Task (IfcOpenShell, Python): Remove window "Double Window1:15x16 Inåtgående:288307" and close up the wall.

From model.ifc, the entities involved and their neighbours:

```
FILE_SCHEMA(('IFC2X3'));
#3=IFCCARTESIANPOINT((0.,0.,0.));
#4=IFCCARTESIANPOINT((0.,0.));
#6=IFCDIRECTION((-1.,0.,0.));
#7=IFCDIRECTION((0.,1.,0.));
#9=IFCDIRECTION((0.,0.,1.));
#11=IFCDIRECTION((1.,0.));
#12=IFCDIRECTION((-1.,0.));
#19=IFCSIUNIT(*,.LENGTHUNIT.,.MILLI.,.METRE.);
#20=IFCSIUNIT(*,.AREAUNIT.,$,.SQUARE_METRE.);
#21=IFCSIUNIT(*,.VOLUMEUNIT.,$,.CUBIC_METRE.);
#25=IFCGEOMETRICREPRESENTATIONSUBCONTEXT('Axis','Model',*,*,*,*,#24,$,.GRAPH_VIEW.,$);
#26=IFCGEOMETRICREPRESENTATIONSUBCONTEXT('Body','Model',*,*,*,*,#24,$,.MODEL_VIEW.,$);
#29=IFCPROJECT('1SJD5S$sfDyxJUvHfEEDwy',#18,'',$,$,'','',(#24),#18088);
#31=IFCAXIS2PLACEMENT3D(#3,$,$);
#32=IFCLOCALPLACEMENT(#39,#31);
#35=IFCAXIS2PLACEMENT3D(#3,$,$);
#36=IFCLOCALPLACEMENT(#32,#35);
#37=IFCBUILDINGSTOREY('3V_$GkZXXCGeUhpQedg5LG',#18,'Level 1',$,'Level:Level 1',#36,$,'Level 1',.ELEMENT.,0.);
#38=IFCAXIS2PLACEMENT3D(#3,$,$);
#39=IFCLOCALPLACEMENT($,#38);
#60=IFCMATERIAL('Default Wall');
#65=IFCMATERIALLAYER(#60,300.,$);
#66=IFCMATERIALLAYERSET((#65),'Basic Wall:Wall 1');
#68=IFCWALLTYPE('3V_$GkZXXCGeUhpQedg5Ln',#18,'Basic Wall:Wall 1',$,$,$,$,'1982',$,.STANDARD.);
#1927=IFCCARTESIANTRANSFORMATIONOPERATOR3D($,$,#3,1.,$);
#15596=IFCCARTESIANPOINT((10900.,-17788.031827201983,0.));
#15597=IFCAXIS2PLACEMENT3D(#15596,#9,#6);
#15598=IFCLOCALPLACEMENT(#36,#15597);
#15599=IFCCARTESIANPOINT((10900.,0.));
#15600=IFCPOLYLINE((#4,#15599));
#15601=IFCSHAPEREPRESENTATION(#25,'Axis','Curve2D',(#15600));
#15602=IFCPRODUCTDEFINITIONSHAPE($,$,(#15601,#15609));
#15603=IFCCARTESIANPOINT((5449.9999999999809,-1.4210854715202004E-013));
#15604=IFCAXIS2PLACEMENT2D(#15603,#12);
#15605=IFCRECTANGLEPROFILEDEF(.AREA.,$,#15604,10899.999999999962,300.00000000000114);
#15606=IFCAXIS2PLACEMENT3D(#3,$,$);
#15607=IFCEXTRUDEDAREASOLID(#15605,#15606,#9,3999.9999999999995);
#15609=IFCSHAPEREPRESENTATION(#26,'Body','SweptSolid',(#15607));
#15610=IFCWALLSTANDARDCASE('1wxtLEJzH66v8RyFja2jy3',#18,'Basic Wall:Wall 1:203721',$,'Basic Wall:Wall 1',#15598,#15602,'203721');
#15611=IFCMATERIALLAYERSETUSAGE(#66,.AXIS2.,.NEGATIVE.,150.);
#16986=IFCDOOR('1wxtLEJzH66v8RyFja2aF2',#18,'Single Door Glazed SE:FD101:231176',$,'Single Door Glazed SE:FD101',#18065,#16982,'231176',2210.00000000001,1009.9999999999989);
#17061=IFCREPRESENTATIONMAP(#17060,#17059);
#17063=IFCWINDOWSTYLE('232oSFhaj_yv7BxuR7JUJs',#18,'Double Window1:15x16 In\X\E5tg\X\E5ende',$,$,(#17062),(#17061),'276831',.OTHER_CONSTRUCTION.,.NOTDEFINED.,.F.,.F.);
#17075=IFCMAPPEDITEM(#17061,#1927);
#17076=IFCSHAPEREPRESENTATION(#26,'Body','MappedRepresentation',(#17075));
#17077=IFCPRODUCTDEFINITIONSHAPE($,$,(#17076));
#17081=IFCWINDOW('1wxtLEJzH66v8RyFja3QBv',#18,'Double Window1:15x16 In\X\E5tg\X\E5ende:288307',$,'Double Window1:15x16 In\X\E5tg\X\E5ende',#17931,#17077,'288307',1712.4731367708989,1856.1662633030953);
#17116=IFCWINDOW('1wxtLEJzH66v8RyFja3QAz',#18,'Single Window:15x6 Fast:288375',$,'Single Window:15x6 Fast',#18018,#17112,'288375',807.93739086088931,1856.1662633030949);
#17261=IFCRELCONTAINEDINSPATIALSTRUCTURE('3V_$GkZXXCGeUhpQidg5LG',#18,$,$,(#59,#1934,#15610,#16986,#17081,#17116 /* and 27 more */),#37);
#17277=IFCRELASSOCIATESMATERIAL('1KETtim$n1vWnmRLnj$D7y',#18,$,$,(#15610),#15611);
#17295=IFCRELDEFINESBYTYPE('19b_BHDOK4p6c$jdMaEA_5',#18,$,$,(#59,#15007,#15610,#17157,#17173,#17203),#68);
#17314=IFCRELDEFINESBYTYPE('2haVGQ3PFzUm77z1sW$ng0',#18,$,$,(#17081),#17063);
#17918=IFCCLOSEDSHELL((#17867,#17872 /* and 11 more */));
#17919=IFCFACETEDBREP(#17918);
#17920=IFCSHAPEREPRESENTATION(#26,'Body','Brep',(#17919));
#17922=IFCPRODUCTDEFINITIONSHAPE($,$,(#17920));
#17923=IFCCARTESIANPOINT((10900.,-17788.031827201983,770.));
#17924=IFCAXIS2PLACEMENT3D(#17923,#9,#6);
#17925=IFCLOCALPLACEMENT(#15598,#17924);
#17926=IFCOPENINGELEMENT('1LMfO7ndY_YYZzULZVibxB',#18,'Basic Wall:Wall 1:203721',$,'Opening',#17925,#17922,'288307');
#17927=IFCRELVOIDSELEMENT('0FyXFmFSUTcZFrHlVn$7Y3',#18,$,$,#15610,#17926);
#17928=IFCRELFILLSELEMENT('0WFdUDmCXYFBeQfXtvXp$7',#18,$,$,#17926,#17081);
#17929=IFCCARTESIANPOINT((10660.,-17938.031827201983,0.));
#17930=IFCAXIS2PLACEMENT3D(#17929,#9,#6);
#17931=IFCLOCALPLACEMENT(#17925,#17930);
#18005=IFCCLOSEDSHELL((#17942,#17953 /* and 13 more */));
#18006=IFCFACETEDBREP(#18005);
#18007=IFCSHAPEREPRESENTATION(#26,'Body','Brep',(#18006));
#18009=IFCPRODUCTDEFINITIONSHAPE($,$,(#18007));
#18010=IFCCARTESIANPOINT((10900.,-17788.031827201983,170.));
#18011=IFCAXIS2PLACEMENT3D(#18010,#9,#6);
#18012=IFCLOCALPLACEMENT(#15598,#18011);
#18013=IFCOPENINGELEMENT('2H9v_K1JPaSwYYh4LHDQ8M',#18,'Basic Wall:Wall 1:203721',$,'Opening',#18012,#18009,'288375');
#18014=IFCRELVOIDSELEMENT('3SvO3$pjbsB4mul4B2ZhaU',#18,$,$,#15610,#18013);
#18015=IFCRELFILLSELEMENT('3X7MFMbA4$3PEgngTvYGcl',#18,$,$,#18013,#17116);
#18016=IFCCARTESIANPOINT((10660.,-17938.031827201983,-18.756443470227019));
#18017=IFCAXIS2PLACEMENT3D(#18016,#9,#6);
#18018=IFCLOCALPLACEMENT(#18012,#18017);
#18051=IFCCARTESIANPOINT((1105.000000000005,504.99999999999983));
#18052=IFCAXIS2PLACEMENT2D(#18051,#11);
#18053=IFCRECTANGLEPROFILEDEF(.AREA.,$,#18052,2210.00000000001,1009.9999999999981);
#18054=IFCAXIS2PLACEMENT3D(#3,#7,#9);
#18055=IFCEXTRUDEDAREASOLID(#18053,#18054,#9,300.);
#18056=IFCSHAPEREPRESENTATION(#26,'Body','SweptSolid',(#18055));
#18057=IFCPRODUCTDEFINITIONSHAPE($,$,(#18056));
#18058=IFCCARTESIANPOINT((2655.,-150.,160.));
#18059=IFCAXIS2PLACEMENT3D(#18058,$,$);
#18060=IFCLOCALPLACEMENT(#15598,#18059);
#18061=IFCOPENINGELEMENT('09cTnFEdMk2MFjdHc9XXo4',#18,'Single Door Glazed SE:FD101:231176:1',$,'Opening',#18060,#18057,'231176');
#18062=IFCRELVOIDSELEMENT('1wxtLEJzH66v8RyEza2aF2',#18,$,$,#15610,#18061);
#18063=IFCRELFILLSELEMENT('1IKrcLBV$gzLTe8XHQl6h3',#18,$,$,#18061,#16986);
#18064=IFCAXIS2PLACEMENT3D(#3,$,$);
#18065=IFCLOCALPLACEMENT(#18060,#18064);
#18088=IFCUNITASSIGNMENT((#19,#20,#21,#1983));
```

```python
import ifcopenshell
import ifcopenshell.api.feature
import ifcopenshell.api.root
import ifcopenshell.geom
import ifcopenshell.util.shape

model = ifcopenshell.open("model.ifc")
settings = ifcopenshell.geom.settings()


def volume(element):
    """Net volume in cubic metres, openings subtracted."""
    shape = ifcopenshell.geom.create_shape(settings, element)
    return ifcopenshell.util.shape.get_volume(shape.geometry)


window = model.by_id(17081)
opening = window.FillsVoids[0].RelatingOpeningElement
wall = opening.VoidsElements[0].RelatingBuildingElement
before = volume(wall)

ifcopenshell.api.root.remove_product(model, product=window)
ifcopenshell.api.feature.remove_feature(model, feature=opening)

after = volume(wall)

print(f"wall volume {before:.3f} -> {after:.3f} m3")

model.write("model_rev.ifc")
```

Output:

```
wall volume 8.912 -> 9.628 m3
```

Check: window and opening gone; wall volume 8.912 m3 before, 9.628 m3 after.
